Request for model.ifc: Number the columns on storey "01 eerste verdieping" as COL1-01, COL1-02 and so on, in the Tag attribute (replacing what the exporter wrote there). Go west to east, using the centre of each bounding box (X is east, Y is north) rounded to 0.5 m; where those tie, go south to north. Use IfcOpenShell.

First a look at what the model holds.

```python
import ifcopenshell
import ifcopenshell.util.element
import ifcopenshell.util.placement

model = ifcopenshell.open("model.ifc")
print(model.schema)
storey = next(s for s in model.by_type("IfcBuildingStorey") if s.Name == "01 eerste verdieping")
columns = [e for e in ifcopenshell.util.element.get_decomposition(storey) if e.is_a("IfcColumn")]
for e in sorted(columns, key=lambda e: e.id()):
    origin = ifcopenshell.util.placement.get_local_placement(e.ObjectPlacement)[:3, 3]
    print(e.id(), e.Tag, e.Name, origin.round(2) + 0.0, sep=" | ")
```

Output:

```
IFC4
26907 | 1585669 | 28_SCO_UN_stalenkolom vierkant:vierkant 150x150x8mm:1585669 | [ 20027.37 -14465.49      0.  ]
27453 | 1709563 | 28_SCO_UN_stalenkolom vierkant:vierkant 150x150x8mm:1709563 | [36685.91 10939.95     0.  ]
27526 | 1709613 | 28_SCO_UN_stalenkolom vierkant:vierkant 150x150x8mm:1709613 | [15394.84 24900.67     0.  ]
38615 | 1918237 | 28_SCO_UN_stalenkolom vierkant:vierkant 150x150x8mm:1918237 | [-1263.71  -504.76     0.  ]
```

```python
import ifcopenshell
import ifcopenshell.geom
import ifcopenshell.util.element
import ifcopenshell.util.shape

model = ifcopenshell.open("model.ifc")
settings = ifcopenshell.geom.settings()
settings.set("use-world-coords", True)


def centre(element):
    shape = ifcopenshell.geom.create_shape(settings, element)
    return ifcopenshell.util.shape.get_bbox_centroid(shape.geometry)


storey = next(s for s in model.by_type("IfcBuildingStorey") if s.Name == "01 eerste verdieping")
columns = [e for e in ifcopenshell.util.element.get_decomposition(storey) if e.is_a("IfcColumn")]

# Insertion points can sit at a corner or the storey origin, so sort by the geometry (in metres).
centres = {e: centre(e) for e in columns}
columns.sort(key=lambda e: (round(centres[e][0] / 0.5), centres[e][1]))

for i, e in enumerate(columns, start=1):
    number = f"COL1-{i:02d}"
    e.Tag = number
    print(e.id(), number)

model.write("model_v2.ifc")
```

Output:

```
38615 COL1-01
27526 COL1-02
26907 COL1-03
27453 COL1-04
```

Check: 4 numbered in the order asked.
